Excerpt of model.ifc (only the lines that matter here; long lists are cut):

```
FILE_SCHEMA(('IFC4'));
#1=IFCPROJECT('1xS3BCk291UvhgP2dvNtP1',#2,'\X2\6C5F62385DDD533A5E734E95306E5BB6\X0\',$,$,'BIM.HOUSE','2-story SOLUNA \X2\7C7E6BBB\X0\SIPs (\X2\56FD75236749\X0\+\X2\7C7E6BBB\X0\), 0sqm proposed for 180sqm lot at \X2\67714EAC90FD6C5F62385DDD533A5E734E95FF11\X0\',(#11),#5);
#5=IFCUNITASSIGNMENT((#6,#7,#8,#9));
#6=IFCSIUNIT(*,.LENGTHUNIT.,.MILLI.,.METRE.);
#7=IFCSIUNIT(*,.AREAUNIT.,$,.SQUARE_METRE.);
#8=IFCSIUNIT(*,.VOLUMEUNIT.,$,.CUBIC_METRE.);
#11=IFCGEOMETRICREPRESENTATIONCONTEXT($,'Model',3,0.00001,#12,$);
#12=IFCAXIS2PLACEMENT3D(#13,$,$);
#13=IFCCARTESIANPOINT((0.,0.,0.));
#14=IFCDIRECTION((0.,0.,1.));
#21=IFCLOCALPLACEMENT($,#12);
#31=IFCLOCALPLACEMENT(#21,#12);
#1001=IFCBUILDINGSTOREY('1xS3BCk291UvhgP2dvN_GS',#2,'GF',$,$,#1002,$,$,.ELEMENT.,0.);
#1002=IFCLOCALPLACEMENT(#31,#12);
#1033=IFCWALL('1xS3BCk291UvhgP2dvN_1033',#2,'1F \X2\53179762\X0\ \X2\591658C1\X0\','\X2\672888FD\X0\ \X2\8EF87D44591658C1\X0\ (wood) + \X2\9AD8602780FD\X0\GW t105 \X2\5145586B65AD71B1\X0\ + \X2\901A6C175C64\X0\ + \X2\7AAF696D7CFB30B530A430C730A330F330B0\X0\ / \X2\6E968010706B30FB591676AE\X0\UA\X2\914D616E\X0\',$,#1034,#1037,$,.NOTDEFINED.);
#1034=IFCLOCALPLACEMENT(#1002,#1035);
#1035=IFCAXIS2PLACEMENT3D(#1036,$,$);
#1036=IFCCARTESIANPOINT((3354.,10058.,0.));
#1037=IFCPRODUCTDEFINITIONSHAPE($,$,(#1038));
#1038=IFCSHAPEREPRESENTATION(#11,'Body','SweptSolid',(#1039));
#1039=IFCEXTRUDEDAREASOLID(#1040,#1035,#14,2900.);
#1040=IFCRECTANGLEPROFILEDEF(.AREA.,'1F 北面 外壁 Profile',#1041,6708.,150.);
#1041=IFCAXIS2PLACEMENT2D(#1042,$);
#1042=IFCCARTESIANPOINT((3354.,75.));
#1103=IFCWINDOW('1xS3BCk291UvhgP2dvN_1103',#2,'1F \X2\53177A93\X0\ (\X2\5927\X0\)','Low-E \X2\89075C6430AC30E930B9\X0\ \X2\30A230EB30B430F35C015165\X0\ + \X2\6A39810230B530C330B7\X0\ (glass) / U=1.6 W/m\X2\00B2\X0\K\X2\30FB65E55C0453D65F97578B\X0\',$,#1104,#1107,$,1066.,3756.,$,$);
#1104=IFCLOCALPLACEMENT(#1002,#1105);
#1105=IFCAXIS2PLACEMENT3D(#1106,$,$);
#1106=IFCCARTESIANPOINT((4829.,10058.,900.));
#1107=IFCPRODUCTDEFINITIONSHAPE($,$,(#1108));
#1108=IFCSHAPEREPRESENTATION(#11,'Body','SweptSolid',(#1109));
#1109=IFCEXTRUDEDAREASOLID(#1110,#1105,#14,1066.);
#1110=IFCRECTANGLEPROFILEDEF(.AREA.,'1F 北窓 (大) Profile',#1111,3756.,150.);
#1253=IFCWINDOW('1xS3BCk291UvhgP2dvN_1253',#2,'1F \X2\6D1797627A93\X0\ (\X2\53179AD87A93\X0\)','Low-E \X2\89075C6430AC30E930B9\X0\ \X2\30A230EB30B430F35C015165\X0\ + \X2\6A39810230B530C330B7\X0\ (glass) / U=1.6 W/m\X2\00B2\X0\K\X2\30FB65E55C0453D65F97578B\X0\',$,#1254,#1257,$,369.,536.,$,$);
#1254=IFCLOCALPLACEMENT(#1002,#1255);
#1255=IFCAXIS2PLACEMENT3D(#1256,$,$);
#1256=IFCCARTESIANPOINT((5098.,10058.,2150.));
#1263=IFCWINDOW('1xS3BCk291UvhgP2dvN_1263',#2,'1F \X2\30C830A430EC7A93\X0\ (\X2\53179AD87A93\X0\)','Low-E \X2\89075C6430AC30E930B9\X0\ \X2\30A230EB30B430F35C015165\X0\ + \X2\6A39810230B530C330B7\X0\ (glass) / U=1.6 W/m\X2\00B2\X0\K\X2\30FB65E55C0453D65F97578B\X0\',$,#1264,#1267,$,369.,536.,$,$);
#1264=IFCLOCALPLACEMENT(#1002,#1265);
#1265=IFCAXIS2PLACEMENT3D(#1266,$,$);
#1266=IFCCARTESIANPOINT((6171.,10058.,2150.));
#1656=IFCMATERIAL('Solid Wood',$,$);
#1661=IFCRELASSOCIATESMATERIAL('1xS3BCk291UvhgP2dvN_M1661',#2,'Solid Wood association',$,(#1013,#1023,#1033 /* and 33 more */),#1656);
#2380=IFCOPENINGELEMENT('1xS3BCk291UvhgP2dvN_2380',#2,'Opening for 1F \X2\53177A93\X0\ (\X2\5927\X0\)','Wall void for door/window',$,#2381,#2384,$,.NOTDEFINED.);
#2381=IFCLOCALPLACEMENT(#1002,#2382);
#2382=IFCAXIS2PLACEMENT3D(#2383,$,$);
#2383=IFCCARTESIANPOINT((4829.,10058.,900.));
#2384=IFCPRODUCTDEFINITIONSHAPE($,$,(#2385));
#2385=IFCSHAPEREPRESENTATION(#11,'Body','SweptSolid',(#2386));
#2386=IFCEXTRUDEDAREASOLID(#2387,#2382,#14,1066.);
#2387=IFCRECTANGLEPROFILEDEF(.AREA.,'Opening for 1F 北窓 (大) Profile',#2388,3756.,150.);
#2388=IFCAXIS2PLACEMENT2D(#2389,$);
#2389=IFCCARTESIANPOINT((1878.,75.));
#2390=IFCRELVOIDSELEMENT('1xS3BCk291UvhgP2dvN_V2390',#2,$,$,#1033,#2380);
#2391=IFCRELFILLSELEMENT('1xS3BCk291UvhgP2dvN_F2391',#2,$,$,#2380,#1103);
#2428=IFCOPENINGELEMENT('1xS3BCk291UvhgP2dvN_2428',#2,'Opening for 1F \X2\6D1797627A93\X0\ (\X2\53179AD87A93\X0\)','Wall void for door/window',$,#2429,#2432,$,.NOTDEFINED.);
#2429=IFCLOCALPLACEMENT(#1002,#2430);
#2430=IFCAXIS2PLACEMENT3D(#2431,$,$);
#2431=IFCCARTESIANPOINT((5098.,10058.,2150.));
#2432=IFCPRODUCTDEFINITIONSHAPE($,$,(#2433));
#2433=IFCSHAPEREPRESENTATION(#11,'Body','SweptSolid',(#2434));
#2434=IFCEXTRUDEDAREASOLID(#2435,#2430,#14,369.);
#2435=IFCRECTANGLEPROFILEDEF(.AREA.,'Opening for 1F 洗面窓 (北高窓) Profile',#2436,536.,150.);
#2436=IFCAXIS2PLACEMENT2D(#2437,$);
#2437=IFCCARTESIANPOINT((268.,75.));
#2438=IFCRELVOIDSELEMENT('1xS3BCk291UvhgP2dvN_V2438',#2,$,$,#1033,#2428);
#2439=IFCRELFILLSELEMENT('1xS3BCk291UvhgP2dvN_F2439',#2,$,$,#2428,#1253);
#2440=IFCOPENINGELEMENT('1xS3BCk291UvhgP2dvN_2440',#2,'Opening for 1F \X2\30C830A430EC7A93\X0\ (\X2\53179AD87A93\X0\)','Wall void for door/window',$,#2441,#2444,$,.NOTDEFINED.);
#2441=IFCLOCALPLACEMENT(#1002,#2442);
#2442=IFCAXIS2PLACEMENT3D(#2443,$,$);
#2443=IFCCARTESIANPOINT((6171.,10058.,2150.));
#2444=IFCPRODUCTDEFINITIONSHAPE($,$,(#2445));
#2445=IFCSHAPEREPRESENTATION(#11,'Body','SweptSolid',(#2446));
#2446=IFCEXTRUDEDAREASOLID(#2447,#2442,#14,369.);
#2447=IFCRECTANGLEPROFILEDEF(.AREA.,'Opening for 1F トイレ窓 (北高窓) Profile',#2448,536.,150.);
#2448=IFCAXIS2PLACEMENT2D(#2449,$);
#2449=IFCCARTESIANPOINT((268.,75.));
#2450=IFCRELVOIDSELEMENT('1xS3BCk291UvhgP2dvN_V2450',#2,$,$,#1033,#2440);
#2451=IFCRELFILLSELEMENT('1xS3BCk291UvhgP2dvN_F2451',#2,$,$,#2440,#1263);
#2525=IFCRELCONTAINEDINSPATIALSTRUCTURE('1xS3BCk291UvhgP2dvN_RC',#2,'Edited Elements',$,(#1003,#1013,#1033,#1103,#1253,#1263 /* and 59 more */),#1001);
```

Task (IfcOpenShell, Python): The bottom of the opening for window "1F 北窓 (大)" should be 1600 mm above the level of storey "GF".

```python
import numpy as np
import ifcopenshell
import ifcopenshell.api.geometry
import ifcopenshell.geom
import ifcopenshell.util.element
import ifcopenshell.util.placement
import ifcopenshell.util.shape
import ifcopenshell.util.unit

model = ifcopenshell.open("model.ifc")
unit_scale = ifcopenshell.util.unit.calculate_unit_scale(model)

window = model.by_guid("1xS3BCk291UvhgP2dvN_1103")
opening = window.FillsVoids[0].RelatingOpeningElement
storey = ifcopenshell.util.element.get_container(window, ifc_class="IfcBuildingStorey")
level = ifcopenshell.util.placement.get_local_placement(storey.ObjectPlacement)[2, 3]

# The opening's origin need not be at the sill, so measure its lowest point.
shape = ifcopenshell.geom.create_shape(ifcopenshell.geom.settings(), opening)
bottom = ifcopenshell.util.shape.get_shape_bottom_elevation(shape, shape.geometry) / unit_scale
dz = level + 1600.0 - bottom

shift = np.array([0.0, 0.0, dz])
# The window is not placed relative to its opening, so move both.
for product in (opening, window):
    matrix = ifcopenshell.util.placement.get_local_placement(product.ObjectPlacement)
    matrix[:3, 3] += shift
    ifcopenshell.api.geometry.edit_object_placement(model, product=product, matrix=matrix, is_si=False)

print(f"moved by {dz * unit_scale:+.3f} m")

model.write("model-out.ifc")
```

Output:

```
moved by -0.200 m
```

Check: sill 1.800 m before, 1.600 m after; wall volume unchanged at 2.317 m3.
